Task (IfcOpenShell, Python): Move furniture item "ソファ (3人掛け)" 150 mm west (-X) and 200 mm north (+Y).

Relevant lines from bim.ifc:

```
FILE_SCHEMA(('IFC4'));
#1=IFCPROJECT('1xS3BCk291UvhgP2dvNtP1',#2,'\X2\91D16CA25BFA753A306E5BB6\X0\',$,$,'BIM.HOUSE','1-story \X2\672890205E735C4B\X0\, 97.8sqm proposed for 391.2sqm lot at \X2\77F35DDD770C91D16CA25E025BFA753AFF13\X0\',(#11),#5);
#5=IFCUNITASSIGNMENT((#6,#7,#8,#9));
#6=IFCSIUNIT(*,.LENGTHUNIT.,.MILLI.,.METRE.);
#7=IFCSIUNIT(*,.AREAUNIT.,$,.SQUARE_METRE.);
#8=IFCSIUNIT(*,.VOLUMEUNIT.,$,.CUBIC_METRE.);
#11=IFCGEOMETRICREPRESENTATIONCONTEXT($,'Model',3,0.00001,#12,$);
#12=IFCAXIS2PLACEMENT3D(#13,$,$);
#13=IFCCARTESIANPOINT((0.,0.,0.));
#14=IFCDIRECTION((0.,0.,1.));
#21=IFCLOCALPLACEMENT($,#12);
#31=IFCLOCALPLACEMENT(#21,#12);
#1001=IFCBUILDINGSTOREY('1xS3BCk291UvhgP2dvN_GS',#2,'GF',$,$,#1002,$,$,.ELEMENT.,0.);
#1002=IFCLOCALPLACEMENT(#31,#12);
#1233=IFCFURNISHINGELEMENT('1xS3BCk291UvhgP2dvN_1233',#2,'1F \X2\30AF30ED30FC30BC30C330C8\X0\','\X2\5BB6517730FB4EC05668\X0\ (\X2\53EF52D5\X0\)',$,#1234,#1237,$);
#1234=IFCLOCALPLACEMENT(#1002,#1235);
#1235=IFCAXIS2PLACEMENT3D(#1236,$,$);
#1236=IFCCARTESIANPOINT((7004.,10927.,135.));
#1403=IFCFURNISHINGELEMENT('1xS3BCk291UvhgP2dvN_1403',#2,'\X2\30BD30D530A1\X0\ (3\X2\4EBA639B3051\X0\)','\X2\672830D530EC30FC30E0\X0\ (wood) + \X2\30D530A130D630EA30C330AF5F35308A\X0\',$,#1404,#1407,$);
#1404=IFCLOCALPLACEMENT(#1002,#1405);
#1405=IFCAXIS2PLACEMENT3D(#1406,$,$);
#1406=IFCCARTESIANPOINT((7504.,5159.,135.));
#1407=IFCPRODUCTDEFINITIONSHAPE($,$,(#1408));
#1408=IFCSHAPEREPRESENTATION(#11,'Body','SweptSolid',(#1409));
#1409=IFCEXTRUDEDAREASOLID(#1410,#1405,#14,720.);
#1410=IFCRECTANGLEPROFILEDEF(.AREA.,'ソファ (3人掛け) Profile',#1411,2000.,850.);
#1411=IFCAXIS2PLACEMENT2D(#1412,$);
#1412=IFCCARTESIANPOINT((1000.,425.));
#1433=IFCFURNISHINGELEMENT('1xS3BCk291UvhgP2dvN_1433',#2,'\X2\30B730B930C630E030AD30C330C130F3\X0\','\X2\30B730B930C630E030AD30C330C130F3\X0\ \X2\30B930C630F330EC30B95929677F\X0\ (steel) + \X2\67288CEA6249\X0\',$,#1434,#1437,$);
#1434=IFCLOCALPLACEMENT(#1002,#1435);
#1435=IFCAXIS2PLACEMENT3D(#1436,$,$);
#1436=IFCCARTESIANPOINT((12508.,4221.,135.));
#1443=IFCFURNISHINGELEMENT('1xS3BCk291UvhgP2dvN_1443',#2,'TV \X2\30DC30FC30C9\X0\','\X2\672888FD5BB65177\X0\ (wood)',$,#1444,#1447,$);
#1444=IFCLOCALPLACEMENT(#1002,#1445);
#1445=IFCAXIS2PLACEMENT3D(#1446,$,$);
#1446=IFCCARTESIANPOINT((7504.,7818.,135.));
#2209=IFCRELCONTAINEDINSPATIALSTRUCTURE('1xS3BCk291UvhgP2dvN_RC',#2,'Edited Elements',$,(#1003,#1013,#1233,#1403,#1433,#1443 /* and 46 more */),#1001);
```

```python
import ifcopenshell
import ifcopenshell.api.geometry
import ifcopenshell.util.placement
import ifcopenshell.util.unit

model = ifcopenshell.open("bim.ifc")
unit_scale = ifcopenshell.util.unit.calculate_unit_scale(model)

item = model.by_guid("1xS3BCk291UvhgP2dvN_1403")
matrix = ifcopenshell.util.placement.get_local_placement(item.ObjectPlacement)
matrix[0, 3] -= 0.15 / unit_scale
matrix[1, 3] += 0.2 / unit_scale
ifcopenshell.api.geometry.edit_object_placement(model, product=item, matrix=matrix, is_si=False)

print(ifcopenshell.util.placement.get_local_placement(item.ObjectPlacement).round(3) + 0.0)

model.write("bim-out.ifc")
```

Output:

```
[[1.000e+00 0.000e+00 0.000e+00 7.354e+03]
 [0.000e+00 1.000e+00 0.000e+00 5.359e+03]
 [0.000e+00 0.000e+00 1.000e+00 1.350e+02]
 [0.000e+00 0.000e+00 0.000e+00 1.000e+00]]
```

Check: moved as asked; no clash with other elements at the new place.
